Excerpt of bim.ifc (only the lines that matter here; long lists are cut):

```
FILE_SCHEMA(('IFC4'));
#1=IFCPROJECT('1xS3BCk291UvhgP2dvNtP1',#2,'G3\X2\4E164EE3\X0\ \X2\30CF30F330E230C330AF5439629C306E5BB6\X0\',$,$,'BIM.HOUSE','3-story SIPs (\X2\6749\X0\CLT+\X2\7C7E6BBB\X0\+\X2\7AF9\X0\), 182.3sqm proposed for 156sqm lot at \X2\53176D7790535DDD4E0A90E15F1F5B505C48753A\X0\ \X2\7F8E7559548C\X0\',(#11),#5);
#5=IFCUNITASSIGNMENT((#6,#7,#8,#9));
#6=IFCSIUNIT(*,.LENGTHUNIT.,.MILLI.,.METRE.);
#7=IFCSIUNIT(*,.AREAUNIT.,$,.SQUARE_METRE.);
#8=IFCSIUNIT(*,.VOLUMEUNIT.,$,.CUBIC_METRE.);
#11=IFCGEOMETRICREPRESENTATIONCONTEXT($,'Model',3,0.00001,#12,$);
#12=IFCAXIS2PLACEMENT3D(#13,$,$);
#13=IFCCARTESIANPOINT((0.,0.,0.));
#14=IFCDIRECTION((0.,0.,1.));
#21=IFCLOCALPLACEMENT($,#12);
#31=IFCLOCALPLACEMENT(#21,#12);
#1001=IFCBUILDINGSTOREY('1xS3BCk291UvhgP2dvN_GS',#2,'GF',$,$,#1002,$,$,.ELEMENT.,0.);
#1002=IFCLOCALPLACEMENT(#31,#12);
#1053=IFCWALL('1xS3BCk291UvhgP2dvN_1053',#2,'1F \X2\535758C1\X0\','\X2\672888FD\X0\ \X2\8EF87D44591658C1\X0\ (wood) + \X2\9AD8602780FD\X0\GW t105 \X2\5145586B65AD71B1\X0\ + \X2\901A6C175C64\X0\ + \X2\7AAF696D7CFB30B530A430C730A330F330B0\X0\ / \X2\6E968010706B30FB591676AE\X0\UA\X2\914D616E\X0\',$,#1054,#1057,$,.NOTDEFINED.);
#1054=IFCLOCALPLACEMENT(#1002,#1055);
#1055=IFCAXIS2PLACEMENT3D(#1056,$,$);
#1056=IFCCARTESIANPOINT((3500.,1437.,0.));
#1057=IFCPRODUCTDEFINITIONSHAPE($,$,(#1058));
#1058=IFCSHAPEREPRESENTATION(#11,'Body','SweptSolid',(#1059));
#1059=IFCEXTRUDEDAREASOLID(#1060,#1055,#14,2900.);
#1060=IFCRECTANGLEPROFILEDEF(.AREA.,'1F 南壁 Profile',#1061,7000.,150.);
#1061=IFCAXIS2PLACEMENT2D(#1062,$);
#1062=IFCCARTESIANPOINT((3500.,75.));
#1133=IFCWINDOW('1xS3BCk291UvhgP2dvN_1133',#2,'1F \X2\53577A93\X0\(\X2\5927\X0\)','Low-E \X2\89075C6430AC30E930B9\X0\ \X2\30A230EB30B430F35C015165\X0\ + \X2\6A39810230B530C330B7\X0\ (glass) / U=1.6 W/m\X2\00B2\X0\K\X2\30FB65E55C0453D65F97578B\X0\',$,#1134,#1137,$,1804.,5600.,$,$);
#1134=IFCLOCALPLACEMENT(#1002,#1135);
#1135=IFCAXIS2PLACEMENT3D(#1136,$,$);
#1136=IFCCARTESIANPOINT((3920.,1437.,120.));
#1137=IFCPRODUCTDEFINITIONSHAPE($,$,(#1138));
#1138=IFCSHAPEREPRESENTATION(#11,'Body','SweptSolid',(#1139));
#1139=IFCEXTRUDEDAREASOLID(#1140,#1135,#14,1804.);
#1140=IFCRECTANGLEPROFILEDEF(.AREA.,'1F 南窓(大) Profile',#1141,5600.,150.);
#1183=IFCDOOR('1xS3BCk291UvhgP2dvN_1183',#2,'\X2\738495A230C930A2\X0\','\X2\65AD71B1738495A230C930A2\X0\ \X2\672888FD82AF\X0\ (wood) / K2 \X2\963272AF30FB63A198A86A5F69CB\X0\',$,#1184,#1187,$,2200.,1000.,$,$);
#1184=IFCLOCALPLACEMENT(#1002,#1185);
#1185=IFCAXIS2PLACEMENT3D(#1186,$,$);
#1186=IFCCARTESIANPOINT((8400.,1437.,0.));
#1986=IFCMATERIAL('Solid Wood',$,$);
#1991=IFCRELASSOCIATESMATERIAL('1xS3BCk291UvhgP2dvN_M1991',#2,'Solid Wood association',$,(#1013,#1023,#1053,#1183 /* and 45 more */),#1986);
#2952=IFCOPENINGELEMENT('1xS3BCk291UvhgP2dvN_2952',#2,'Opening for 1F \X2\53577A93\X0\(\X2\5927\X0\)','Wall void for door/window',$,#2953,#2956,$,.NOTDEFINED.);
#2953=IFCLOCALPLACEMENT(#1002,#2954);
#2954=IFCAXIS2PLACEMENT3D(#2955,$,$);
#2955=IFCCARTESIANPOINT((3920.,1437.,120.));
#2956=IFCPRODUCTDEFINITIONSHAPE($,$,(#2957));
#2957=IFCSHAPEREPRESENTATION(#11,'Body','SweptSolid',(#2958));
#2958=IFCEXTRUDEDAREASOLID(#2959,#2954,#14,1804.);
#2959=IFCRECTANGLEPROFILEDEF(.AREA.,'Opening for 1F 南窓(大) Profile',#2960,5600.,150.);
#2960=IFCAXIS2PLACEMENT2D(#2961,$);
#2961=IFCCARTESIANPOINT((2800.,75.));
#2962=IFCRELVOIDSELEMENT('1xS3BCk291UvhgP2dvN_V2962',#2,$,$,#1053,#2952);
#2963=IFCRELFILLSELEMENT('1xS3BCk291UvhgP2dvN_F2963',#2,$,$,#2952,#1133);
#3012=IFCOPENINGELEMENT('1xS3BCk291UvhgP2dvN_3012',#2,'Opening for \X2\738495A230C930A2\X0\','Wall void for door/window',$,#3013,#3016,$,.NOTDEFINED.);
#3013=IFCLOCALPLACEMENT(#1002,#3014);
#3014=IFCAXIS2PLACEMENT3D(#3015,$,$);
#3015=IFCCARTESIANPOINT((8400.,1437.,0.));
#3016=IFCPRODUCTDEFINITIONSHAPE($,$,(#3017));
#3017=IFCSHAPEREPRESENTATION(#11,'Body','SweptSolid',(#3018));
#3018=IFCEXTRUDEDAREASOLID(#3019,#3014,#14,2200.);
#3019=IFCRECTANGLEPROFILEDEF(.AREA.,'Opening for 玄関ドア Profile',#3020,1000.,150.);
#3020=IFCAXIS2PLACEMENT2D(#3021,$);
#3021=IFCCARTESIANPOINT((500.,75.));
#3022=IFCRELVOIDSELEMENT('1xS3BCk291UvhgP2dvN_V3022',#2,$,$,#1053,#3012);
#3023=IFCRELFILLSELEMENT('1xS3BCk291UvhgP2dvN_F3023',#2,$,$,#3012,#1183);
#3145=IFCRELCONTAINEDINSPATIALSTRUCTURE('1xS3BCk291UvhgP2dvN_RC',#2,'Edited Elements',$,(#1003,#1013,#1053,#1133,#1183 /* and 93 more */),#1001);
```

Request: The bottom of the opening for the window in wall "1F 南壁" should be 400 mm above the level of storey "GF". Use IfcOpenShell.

```python
import numpy as np
import ifcopenshell
import ifcopenshell.api.geometry
import ifcopenshell.geom
import ifcopenshell.util.element
import ifcopenshell.util.placement
import ifcopenshell.util.shape
import ifcopenshell.util.unit

model = ifcopenshell.open("bim.ifc")
unit_scale = ifcopenshell.util.unit.calculate_unit_scale(model)

window = model.by_guid("1xS3BCk291UvhgP2dvN_1133")
opening = window.FillsVoids[0].RelatingOpeningElement
storey = ifcopenshell.util.element.get_container(window, ifc_class="IfcBuildingStorey")
level = ifcopenshell.util.placement.get_local_placement(storey.ObjectPlacement)[2, 3]

# The opening's origin need not be at the sill, so measure its lowest point.
shape = ifcopenshell.geom.create_shape(ifcopenshell.geom.settings(), opening)
bottom = ifcopenshell.util.shape.get_shape_bottom_elevation(shape, shape.geometry) / unit_scale
dz = level + 0.4 / unit_scale - bottom

shift = np.array([0.0, 0.0, dz])
# The window is not placed relative to its opening, so move both.
for product in (opening, window):
    matrix = ifcopenshell.util.placement.get_local_placement(product.ObjectPlacement)
    matrix[:3, 3] += shift
    ifcopenshell.api.geometry.edit_object_placement(model, product=product, matrix=matrix, is_si=False)

print(f"moved by {dz * unit_scale:+.3f} m")

model.write("bim_edited.ifc")
```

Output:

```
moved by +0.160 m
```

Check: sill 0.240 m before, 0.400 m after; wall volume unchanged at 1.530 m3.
